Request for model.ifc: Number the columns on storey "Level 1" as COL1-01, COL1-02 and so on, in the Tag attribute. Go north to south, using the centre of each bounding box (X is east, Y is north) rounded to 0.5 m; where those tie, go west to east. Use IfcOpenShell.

First a look at what the model holds.

```python
import ifcopenshell
import ifcopenshell.util.element
import ifcopenshell.util.placement

model = ifcopenshell.open("model.ifc")
print(model.schema)
storey = next(s for s in model.by_type("IfcBuildingStorey") if s.Name == "Level 1")
columns = [e for e in ifcopenshell.util.element.get_decomposition(storey) if e.is_a("IfcColumn")]
for e in sorted(columns, key=lambda e: e.id()):
    origin = ifcopenshell.util.placement.get_local_placement(e.ObjectPlacement)[:3, 3]
    print(e.id(), e.Tag, e.Name, origin.round(2) + 0.0, sep=" | ")
```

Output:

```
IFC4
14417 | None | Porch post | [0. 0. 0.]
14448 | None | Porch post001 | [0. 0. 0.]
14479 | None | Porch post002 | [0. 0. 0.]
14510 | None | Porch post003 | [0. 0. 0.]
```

```python
import ifcopenshell
import ifcopenshell.geom
import ifcopenshell.util.element
import ifcopenshell.util.shape

model = ifcopenshell.open("model.ifc")
settings = ifcopenshell.geom.settings()
settings.set("use-world-coords", True)


def centre(element):
    shape = ifcopenshell.geom.create_shape(settings, element)
    return ifcopenshell.util.shape.get_bbox_centroid(shape.geometry)


storey = next(s for s in model.by_type("IfcBuildingStorey") if s.Name == "Level 1")
columns = [e for e in ifcopenshell.util.element.get_decomposition(storey) if e.is_a("IfcColumn")]

# Insertion points can sit at a corner or the storey origin, so sort by the geometry (in metres).
centres = {e: centre(e) for e in columns}
columns.sort(key=lambda e: (-round(centres[e][1] / 0.5), centres[e][0]))

for i, e in enumerate(columns, start=1):
    number = f"COL1-{i:02d}"
    e.Tag = number
    print(e.id(), number)

model.write("model-out.ifc")
```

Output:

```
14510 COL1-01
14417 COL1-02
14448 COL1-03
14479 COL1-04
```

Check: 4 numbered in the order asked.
